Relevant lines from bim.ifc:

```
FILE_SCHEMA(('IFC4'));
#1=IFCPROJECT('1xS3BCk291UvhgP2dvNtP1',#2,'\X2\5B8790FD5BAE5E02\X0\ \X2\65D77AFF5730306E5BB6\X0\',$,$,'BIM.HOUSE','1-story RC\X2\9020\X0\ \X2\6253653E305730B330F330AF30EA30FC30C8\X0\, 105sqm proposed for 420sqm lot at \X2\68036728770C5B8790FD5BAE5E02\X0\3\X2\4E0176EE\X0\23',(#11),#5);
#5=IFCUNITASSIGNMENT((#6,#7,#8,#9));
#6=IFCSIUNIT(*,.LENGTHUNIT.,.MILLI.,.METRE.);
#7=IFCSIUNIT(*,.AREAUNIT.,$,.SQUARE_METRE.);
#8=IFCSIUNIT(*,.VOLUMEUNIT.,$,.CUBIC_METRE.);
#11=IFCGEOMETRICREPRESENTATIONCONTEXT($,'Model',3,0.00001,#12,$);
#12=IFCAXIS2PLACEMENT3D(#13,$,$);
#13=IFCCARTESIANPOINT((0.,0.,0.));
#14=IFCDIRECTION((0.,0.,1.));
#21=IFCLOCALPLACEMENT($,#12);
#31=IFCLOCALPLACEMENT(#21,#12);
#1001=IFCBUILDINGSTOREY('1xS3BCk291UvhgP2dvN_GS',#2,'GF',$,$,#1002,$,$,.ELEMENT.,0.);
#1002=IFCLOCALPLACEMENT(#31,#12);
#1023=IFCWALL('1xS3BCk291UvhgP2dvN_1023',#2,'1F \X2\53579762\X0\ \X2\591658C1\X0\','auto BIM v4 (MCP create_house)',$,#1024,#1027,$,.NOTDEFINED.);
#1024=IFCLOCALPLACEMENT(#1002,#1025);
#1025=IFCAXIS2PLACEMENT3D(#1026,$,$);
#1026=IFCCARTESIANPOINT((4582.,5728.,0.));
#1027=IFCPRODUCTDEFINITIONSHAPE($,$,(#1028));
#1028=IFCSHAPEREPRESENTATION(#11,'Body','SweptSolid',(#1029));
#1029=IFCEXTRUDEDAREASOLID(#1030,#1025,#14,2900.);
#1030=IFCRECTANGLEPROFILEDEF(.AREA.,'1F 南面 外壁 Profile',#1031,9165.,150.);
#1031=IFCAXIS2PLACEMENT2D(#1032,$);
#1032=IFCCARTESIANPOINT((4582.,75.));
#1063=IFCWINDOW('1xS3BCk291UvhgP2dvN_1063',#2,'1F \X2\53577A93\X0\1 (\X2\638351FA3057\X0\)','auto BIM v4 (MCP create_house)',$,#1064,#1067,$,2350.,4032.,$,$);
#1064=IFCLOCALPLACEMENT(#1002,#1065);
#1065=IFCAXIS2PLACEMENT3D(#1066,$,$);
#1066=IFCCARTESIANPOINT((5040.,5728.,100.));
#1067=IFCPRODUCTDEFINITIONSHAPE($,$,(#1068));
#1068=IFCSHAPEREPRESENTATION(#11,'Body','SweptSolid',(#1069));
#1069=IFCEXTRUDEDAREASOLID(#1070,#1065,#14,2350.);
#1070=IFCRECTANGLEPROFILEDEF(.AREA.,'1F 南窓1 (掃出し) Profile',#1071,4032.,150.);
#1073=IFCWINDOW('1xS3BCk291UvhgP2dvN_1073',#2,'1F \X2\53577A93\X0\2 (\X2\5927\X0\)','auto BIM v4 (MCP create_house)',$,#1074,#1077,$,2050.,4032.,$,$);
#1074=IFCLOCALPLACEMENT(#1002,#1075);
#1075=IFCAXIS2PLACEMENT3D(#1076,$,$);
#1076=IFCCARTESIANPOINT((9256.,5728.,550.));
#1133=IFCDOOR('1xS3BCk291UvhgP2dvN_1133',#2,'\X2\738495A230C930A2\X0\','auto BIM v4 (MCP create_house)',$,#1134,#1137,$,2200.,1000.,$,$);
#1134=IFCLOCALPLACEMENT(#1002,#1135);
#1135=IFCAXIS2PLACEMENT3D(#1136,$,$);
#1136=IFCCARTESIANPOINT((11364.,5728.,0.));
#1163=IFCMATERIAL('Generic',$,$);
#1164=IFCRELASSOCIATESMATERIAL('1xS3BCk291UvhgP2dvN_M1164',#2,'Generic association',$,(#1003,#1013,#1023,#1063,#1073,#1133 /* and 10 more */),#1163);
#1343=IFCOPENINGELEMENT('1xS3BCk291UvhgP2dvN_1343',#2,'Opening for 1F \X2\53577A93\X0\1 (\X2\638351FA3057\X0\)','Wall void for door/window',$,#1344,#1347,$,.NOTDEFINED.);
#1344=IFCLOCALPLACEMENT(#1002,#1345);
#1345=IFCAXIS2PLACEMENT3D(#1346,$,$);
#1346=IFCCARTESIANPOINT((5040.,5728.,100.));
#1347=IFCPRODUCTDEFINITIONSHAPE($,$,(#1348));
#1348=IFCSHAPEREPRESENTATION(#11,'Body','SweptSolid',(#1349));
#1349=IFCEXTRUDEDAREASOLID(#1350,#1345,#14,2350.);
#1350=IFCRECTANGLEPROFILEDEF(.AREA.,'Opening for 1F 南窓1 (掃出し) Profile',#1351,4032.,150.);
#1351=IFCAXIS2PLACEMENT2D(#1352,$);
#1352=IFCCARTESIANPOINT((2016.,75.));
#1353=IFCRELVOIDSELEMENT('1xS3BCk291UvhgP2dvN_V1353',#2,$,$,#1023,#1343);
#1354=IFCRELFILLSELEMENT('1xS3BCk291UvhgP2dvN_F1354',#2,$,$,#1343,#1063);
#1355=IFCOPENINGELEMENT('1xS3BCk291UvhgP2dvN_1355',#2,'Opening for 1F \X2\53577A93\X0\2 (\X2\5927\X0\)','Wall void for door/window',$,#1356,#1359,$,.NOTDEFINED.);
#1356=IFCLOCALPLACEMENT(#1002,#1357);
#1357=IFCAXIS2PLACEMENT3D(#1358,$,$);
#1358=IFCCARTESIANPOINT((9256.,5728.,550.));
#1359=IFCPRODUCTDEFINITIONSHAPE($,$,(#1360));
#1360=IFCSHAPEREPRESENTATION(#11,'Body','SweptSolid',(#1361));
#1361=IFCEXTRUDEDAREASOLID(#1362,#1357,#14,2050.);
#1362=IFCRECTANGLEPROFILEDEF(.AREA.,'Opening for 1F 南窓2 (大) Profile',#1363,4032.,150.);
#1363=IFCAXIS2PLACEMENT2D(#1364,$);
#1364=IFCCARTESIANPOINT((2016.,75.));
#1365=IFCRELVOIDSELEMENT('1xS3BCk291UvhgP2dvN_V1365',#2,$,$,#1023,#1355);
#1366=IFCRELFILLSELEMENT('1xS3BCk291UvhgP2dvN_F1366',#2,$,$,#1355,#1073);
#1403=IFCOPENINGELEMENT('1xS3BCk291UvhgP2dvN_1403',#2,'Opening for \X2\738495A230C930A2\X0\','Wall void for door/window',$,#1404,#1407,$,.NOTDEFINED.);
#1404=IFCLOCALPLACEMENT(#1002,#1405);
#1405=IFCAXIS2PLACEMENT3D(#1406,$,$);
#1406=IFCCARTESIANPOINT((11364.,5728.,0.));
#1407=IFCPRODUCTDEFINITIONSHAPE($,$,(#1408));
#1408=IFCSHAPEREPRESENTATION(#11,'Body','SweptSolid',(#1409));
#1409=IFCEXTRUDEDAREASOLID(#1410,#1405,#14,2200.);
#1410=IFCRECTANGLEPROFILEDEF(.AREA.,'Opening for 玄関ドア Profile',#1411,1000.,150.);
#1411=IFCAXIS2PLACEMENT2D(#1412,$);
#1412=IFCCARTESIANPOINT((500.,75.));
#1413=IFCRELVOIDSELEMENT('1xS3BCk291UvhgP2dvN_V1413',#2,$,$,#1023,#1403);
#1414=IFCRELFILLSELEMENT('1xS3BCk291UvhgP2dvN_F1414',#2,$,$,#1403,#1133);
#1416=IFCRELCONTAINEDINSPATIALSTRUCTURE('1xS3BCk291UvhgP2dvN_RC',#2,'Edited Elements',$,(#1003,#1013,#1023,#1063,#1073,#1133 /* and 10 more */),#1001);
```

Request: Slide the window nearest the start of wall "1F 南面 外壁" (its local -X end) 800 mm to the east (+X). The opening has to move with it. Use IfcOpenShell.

```python
import ifcopenshell
import ifcopenshell.api.geometry
import ifcopenshell.util.placement

model = ifcopenshell.open("bim.ifc")

window = model.by_id(1063)
opening = window.FillsVoids[0].RelatingOpeningElement
wall = opening.VoidsElements[0].RelatingBuildingElement

wall_matrix = ifcopenshell.util.placement.get_local_placement(wall.ObjectPlacement)
shift = wall_matrix[:3, 0] * 800.0
before = ifcopenshell.util.placement.get_local_placement(window.ObjectPlacement)[:3, 3].copy()

# The window is not placed relative to its opening, so move both.
for product in (opening, window):
    matrix = ifcopenshell.util.placement.get_local_placement(product.ObjectPlacement)
    matrix[:3, 3] += shift
    ifcopenshell.api.geometry.edit_object_placement(model, product=product, matrix=matrix, is_si=False)

after = ifcopenshell.util.placement.get_local_placement(window.ObjectPlacement)[:3, 3]
print("window moved by", (after - before).round(3) + 0.0)

model.write("bim-out.ifc")
```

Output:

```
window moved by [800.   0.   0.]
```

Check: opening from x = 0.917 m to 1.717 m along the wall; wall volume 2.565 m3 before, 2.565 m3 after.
